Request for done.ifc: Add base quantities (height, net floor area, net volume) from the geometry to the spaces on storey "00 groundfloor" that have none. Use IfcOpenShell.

First a look at what the model holds.

```python
import ifcopenshell
import ifcopenshell.util.element
import ifcopenshell.util.unit

model = ifcopenshell.open("done.ifc")
print(model.schema)
for unit_type in ("LENGTHUNIT", "AREAUNIT", "VOLUMEUNIT"):
    print(unit_type, ifcopenshell.util.unit.calculate_unit_scale(model, unit_type))
storey = next(s for s in model.by_type("IfcBuildingStorey") if s.Name == "00 groundfloor")
spaces = [e for e in ifcopenshell.util.element.get_decomposition(storey) if e.is_a("IfcSpace")]
for e in sorted(spaces, key=lambda e: e.id()):
    print(e.id(), e.is_a(), e.Name, list(ifcopenshell.util.element.get_psets(e, qtos_only=True)), sep=" | ")
```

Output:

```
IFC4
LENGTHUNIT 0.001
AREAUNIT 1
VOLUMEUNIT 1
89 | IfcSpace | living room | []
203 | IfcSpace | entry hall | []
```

```python
import ifcopenshell
import ifcopenshell.api.pset
import ifcopenshell.geom
import ifcopenshell.util.element
import ifcopenshell.util.shape
import ifcopenshell.util.unit

model = ifcopenshell.open("done.ifc")
unit_scale = ifcopenshell.util.unit.calculate_unit_scale(model)
area_scale = ifcopenshell.util.unit.calculate_unit_scale(model, "AREAUNIT")
volume_scale = ifcopenshell.util.unit.calculate_unit_scale(model, "VOLUMEUNIT")
settings = ifcopenshell.geom.settings()

storey = next(s for s in model.by_type("IfcBuildingStorey") if s.Name == "00 groundfloor")
spaces = [e for e in ifcopenshell.util.element.get_decomposition(storey) if e.is_a("IfcSpace")]

for e in sorted(spaces, key=lambda e: e.id()):
    if ifcopenshell.util.element.get_psets(e, qtos_only=True, should_inherit=False):
        continue
    # Geometry comes back in metres, in the element's own axes.
    shape = ifcopenshell.geom.create_shape(settings, e)
    values = {
        "Height": ifcopenshell.util.shape.get_z(shape.geometry) / unit_scale,
        "NetFloorArea": ifcopenshell.util.shape.get_footprint_area(shape.geometry) / area_scale,
        "NetVolume": ifcopenshell.util.shape.get_volume(shape.geometry) / volume_scale,
    }
    qto = ifcopenshell.api.pset.add_qto(model, product=e, name="Qto_SpaceBaseQuantities")
    ifcopenshell.api.pset.edit_qto(model, qto=qto, properties=values)
    print(e.id(), {k: round(v, 3) for k, v in values.items()})

model.write("done_v2.ifc")
```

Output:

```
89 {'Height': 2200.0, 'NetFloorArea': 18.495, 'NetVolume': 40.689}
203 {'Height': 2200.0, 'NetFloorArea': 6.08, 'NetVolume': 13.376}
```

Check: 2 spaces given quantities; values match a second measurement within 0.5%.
